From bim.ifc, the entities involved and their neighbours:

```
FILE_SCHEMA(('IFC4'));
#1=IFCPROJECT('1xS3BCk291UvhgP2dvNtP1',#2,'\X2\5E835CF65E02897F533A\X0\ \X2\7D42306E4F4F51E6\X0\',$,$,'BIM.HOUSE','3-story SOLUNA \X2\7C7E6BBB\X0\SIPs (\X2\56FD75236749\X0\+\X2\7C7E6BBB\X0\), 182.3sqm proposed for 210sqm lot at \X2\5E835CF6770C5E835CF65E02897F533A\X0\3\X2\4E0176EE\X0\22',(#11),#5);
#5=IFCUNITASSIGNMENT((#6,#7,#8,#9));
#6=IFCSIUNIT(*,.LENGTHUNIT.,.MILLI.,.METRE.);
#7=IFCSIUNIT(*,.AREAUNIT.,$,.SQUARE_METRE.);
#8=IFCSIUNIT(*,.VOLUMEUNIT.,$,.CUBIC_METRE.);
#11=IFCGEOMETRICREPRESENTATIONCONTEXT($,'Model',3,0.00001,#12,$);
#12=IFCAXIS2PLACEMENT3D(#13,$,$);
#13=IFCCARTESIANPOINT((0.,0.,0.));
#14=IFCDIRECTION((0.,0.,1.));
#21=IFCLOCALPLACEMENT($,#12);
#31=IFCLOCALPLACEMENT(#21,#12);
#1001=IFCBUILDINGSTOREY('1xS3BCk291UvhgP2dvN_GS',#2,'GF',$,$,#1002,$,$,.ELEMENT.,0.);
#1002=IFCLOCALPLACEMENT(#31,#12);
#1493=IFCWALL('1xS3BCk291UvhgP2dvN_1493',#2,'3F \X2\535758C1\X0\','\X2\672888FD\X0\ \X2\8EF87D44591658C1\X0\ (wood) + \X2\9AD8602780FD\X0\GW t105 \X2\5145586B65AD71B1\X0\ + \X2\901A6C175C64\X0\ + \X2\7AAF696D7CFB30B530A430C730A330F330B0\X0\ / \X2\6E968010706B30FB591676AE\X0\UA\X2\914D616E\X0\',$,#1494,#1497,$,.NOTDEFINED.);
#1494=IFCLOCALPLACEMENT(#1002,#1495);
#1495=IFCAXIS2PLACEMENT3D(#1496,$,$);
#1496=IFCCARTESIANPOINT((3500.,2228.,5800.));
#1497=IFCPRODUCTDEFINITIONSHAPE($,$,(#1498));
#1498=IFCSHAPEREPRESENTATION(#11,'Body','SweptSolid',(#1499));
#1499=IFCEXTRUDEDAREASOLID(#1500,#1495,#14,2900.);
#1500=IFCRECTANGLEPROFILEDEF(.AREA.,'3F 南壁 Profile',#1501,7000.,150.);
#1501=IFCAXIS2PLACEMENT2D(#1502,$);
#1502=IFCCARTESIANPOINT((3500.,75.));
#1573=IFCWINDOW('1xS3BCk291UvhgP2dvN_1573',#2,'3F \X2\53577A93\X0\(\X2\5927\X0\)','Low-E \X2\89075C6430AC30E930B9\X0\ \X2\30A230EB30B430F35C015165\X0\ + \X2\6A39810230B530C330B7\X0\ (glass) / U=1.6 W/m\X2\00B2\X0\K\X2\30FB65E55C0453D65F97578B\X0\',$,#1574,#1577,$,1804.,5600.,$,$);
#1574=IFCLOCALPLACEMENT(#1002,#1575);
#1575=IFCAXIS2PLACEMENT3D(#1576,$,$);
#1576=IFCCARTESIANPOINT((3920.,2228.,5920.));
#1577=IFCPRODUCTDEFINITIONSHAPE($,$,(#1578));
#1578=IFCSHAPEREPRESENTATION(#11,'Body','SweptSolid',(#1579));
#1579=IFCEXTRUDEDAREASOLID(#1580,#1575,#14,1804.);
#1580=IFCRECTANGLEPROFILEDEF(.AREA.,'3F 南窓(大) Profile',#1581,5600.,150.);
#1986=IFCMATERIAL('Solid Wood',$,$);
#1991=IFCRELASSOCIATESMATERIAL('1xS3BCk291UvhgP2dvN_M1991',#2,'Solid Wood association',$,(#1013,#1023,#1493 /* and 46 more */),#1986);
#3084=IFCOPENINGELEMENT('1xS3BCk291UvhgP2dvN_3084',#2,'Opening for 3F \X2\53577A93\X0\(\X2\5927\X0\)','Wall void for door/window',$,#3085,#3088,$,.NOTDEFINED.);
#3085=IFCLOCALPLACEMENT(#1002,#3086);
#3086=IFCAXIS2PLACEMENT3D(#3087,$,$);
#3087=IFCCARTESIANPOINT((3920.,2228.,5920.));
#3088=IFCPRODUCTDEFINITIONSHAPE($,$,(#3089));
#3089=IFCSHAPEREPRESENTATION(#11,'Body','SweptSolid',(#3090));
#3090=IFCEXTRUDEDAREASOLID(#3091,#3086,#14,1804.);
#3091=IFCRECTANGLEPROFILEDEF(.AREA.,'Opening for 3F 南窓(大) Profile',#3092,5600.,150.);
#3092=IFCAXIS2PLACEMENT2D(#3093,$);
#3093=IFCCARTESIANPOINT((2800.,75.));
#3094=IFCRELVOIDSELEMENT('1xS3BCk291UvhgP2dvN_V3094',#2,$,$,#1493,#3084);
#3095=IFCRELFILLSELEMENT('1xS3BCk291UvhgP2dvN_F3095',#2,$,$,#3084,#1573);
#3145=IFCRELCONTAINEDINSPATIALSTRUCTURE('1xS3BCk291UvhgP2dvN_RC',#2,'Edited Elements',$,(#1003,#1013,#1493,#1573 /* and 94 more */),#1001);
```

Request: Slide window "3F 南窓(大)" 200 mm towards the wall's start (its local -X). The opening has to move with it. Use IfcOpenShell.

```python
import ifcopenshell
import ifcopenshell.api.geometry
import ifcopenshell.util.placement
import ifcopenshell.util.unit

model = ifcopenshell.open("bim.ifc")
unit_scale = ifcopenshell.util.unit.calculate_unit_scale(model)

window = model.by_guid("1xS3BCk291UvhgP2dvN_1573")
opening = window.FillsVoids[0].RelatingOpeningElement
wall = opening.VoidsElements[0].RelatingBuildingElement

wall_matrix = ifcopenshell.util.placement.get_local_placement(wall.ObjectPlacement)
shift = wall_matrix[:3, 0] * -0.2 / unit_scale
before = ifcopenshell.util.placement.get_local_placement(window.ObjectPlacement)[:3, 3].copy()

# The window is not placed relative to its opening, so move both.
for product in (opening, window):
    matrix = ifcopenshell.util.placement.get_local_placement(product.ObjectPlacement)
    matrix[:3, 3] += shift
    ifcopenshell.api.geometry.edit_object_placement(model, product=product, matrix=matrix, is_si=False)

after = ifcopenshell.util.placement.get_local_placement(window.ObjectPlacement)[:3, 3]
print("window moved by", (after - before).round(3) + 0.0)

model.write("bim_v2.ifc")
```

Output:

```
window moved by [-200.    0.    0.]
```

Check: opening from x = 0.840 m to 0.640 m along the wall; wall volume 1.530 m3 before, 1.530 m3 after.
